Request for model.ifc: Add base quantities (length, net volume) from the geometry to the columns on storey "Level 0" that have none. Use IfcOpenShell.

First a look at what the model holds.

```python
import ifcopenshell
import ifcopenshell.util.element
import ifcopenshell.util.unit

model = ifcopenshell.open("model.ifc")
print(model.schema)
for unit_type in ("LENGTHUNIT", "AREAUNIT", "VOLUMEUNIT"):
    print(unit_type, ifcopenshell.util.unit.calculate_unit_scale(model, unit_type))
storey = next(s for s in model.by_type("IfcBuildingStorey") if s.Name == "Level 0")
columns = [e for e in ifcopenshell.util.element.get_decomposition(storey) if e.is_a("IfcColumn")]
for e in sorted(columns, key=lambda e: e.id()):
    print(e.id(), e.is_a(), e.Name, list(ifcopenshell.util.element.get_psets(e, qtos_only=True)), sep=" | ")
```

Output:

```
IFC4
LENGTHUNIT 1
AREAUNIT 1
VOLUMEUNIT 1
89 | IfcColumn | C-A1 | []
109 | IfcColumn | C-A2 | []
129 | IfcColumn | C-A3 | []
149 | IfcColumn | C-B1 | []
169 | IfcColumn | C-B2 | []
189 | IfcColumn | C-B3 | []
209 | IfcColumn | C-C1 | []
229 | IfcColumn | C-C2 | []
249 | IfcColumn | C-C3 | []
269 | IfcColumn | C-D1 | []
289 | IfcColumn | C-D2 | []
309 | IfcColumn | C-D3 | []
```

```python
import ifcopenshell
import ifcopenshell.api.pset
import ifcopenshell.geom
import ifcopenshell.util.element
import ifcopenshell.util.shape
import ifcopenshell.util.unit

model = ifcopenshell.open("model.ifc")
unit_scale = ifcopenshell.util.unit.calculate_unit_scale(model)
volume_scale = ifcopenshell.util.unit.calculate_unit_scale(model, "VOLUMEUNIT")
settings = ifcopenshell.geom.settings()

storey = next(s for s in model.by_type("IfcBuildingStorey") if s.Name == "Level 0")
columns = [e for e in ifcopenshell.util.element.get_decomposition(storey) if e.is_a("IfcColumn")]

for e in sorted(columns, key=lambda e: e.id()):
    if ifcopenshell.util.element.get_psets(e, qtos_only=True, should_inherit=False):
        continue
    # Geometry comes back in metres, in the element's own axes.
    shape = ifcopenshell.geom.create_shape(settings, e)
    values = {
        "Length": ifcopenshell.util.shape.get_z(shape.geometry) / unit_scale,
        "NetVolume": ifcopenshell.util.shape.get_volume(shape.geometry) / volume_scale,
    }
    qto = ifcopenshell.api.pset.add_qto(model, product=e, name="Qto_ColumnBaseQuantities")
    ifcopenshell.api.pset.edit_qto(model, qto=qto, properties=values)
    print(e.id(), {k: round(v, 3) for k, v in values.items()})

model.write("model-out.ifc")
```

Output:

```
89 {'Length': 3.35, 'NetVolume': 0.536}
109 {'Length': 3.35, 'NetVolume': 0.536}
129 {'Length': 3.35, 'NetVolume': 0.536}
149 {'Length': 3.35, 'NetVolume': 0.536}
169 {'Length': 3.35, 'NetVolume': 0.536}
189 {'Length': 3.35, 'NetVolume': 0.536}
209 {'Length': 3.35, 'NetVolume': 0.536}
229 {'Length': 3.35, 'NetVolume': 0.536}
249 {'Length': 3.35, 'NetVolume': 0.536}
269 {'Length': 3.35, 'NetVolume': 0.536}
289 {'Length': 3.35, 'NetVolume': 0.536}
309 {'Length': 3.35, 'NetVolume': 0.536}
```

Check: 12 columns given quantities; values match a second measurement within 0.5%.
